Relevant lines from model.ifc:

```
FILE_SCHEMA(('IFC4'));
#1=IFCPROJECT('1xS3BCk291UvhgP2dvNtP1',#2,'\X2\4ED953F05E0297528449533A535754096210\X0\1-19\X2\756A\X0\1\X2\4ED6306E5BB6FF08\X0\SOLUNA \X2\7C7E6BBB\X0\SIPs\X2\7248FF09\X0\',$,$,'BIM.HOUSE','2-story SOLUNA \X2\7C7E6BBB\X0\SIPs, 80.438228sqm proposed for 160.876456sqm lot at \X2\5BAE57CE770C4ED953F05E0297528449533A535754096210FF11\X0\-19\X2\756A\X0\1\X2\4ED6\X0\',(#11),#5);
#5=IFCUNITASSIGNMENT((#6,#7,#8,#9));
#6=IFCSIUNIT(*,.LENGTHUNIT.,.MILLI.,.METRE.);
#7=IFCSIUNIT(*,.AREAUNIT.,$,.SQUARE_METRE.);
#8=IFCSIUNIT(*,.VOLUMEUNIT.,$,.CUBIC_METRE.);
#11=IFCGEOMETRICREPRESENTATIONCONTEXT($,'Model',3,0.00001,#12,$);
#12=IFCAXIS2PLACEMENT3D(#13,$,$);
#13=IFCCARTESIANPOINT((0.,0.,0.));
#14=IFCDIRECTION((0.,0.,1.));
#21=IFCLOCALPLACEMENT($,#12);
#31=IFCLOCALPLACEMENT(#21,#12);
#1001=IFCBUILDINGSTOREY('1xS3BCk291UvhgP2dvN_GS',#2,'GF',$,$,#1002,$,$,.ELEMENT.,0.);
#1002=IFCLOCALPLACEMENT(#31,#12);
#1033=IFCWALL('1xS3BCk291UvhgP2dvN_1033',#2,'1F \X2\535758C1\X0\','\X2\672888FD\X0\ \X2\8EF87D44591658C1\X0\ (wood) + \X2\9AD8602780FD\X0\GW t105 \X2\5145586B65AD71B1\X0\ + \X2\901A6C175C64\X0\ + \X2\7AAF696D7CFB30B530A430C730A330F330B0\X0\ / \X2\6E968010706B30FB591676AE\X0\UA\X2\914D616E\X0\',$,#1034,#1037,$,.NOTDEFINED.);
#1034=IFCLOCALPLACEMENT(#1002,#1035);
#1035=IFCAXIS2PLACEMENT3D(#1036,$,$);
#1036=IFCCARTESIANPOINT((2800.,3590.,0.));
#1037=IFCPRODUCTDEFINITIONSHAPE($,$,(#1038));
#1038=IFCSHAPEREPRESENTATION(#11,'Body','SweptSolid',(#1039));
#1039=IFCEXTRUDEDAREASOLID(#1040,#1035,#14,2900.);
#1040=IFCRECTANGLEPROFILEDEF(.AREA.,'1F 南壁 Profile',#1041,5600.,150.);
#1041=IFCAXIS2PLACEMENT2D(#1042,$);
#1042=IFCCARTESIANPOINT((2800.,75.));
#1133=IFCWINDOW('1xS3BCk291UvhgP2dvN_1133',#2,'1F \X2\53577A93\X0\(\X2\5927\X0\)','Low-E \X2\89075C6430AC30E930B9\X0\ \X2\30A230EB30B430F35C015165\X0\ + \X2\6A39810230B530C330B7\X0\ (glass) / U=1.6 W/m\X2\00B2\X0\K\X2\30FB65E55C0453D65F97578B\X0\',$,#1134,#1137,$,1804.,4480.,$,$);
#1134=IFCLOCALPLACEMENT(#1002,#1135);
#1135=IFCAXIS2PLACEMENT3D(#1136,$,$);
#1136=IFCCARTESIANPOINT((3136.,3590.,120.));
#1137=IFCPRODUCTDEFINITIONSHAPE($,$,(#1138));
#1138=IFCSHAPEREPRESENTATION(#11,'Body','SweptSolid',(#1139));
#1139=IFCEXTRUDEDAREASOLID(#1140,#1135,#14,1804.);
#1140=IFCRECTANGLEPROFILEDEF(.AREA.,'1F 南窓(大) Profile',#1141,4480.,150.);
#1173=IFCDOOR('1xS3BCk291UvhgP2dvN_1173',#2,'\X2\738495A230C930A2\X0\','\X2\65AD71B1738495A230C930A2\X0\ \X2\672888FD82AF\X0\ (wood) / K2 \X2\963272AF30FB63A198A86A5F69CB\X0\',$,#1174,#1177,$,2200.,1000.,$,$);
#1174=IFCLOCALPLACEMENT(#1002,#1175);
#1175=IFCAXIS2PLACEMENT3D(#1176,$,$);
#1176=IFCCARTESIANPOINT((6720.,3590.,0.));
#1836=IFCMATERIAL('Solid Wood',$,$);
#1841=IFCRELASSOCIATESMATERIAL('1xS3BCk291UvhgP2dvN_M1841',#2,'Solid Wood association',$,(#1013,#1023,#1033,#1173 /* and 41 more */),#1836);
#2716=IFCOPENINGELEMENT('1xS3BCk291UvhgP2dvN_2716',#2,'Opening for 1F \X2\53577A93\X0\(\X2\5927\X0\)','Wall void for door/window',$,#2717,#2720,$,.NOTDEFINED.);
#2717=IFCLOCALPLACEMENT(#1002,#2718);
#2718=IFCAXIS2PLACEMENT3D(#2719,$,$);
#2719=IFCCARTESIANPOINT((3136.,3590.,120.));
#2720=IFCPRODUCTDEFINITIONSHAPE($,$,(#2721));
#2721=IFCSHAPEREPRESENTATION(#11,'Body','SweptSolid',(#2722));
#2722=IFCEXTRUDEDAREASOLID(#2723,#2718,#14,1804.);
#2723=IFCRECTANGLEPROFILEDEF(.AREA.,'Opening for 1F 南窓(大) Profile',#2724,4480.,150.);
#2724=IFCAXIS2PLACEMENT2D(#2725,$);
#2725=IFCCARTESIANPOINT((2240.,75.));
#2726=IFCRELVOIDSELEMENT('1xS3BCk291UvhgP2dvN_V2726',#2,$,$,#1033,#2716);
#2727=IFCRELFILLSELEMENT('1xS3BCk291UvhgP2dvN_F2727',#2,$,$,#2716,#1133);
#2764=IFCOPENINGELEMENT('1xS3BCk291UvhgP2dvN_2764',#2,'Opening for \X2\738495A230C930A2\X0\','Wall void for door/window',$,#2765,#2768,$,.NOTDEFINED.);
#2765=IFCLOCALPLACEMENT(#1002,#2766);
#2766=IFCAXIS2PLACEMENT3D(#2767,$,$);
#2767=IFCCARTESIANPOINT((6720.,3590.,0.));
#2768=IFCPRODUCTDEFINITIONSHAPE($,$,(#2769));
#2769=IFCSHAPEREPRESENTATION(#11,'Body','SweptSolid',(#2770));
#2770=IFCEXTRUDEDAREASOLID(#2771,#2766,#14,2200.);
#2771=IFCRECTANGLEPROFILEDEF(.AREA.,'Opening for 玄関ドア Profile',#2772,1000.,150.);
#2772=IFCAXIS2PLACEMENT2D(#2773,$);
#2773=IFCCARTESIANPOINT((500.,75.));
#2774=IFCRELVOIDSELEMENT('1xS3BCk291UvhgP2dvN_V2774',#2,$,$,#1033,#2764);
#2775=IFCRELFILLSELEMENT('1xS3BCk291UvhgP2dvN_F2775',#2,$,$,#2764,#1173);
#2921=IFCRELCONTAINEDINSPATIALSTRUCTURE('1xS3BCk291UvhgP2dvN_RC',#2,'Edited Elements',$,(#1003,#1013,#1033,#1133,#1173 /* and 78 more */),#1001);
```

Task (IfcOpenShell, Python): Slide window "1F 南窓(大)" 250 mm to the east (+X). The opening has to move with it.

```python
import ifcopenshell
import ifcopenshell.api.geometry
import ifcopenshell.util.placement
import ifcopenshell.util.unit

model = ifcopenshell.open("model.ifc")
unit_scale = ifcopenshell.util.unit.calculate_unit_scale(model)

window = model.by_guid("1xS3BCk291UvhgP2dvN_1133")
opening = window.FillsVoids[0].RelatingOpeningElement
wall = opening.VoidsElements[0].RelatingBuildingElement

wall_matrix = ifcopenshell.util.placement.get_local_placement(wall.ObjectPlacement)
shift = wall_matrix[:3, 0] * 0.25 / unit_scale
before = ifcopenshell.util.placement.get_local_placement(window.ObjectPlacement)[:3, 3].copy()

# The window is not placed relative to its opening, so move both.
for product in (opening, window):
    matrix = ifcopenshell.util.placement.get_local_placement(product.ObjectPlacement)
    matrix[:3, 3] += shift
    ifcopenshell.api.geometry.edit_object_placement(model, product=product, matrix=matrix, is_si=False)

after = ifcopenshell.util.placement.get_local_placement(window.ObjectPlacement)[:3, 3]
print("window moved by", (after - before).round(3) + 0.0)

model.write("model_edited.ifc")
```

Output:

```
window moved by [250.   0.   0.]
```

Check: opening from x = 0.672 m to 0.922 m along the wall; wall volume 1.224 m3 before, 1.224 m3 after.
